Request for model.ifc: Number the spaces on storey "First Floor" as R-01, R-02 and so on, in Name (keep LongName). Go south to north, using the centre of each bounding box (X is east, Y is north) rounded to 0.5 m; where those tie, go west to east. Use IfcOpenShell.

First a look at what the model holds.

```python
import ifcopenshell
import ifcopenshell.util.element
import ifcopenshell.util.placement

model = ifcopenshell.open("model.ifc")
print(model.schema)
storey = next(s for s in model.by_type("IfcBuildingStorey") if s.Name == "First Floor")
spaces = [e for e in ifcopenshell.util.element.get_decomposition(storey) if e.is_a("IfcSpace")]
for e in sorted(spaces, key=lambda e: e.id()):
    origin = ifcopenshell.util.placement.get_local_placement(e.ObjectPlacement)[:3, 3]
    print(e.id(), e.Name, e.LongName, origin.round(2) + 0.0, sep=" | ")
```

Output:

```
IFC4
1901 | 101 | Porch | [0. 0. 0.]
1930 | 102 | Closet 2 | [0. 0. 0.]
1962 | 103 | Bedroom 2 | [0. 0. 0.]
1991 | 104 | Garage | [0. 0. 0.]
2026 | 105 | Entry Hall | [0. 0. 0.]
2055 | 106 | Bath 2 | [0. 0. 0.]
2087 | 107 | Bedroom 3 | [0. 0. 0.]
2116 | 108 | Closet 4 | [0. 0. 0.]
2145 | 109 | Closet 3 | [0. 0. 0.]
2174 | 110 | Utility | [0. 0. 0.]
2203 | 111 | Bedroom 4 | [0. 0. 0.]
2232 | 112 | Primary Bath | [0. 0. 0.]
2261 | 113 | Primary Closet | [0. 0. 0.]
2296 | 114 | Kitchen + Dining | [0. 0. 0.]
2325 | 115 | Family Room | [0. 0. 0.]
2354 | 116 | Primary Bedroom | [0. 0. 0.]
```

```python
import ifcopenshell
import ifcopenshell.geom
import ifcopenshell.util.element
import ifcopenshell.util.shape

model = ifcopenshell.open("model.ifc")
settings = ifcopenshell.geom.settings()
settings.set("use-world-coords", True)


def centre(element):
    shape = ifcopenshell.geom.create_shape(settings, element)
    return ifcopenshell.util.shape.get_bbox_centroid(shape.geometry)


storey = next(s for s in model.by_type("IfcBuildingStorey") if s.Name == "First Floor")
spaces = [e for e in ifcopenshell.util.element.get_decomposition(storey) if e.is_a("IfcSpace")]

# Insertion points can sit at a corner or the storey origin, so sort by the geometry (in metres).
centres = {e: centre(e) for e in spaces}
spaces.sort(key=lambda e: (round(centres[e][1] / 0.5), centres[e][0]))

for i, e in enumerate(spaces, start=1):
    number = f"R-{i:02d}"
    e.Name = number
    print(e.id(), number)

model.write("model_rev.ifc")
```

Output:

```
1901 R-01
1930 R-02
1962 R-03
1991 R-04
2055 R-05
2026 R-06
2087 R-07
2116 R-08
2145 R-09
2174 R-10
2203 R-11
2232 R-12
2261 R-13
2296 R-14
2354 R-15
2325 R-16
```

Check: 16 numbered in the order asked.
